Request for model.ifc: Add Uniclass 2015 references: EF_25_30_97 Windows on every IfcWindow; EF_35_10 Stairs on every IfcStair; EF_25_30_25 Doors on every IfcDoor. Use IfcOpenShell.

First a look at what the model holds.

```python
import ifcopenshell

model = ifcopenshell.open("model.ifc")
print(model.schema)
print("classifications:", [c.Name for c in model.by_type("IfcClassification")])
for ifc_class in ("IfcDoor", "IfcRoof", "IfcStair", "IfcWall", "IfcWindow"):
    print(ifc_class, len(model.by_type(ifc_class)))
```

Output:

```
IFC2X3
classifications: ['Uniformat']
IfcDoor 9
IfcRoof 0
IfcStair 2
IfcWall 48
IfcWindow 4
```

```python
import ifcopenshell
import ifcopenshell.api.classification

model = ifcopenshell.open("model.ifc")

# IFC2X3 requires Source and Edition and has no link from the project to the system.
system = model.create_entity("IfcClassification", Source="NBS", Edition="2015", Name="Uniclass 2015")

codes = {
    "IfcWindow": ("EF_25_30_97", "Windows"),
    "IfcStair": ("EF_35_10", "Stairs"),
    "IfcDoor": ("EF_25_30_25", "Doors"),
}
for ifc_class, (code, name) in codes.items():
    products = model.by_type(ifc_class)
    ifcopenshell.api.classification.add_reference(
        model, products=products, classification=system, identification=code, name=name
    )
    print(code, len(products))

model.write("model_rev.ifc")
```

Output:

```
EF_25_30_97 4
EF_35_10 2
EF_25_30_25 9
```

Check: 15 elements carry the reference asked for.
